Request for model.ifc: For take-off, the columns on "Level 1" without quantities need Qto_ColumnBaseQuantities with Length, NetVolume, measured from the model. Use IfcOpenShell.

First a look at what the model holds.

```python
import ifcopenshell
import ifcopenshell.util.element
import ifcopenshell.util.unit

model = ifcopenshell.open("model.ifc")
print(model.schema)
for unit_type in ("LENGTHUNIT", "AREAUNIT", "VOLUMEUNIT"):
    print(unit_type, ifcopenshell.util.unit.calculate_unit_scale(model, unit_type))
storey = next(s for s in model.by_type("IfcBuildingStorey") if s.Name == "Level 1")
columns = [e for e in ifcopenshell.util.element.get_decomposition(storey) if e.is_a("IfcColumn")]
for e in sorted(columns, key=lambda e: e.id()):
    print(e.id(), e.is_a(), e.Name, list(ifcopenshell.util.element.get_psets(e, qtos_only=True)), sep=" | ")
```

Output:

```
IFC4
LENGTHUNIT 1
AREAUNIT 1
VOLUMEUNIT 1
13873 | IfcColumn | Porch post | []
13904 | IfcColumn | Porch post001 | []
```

```python
import ifcopenshell
import ifcopenshell.api.pset
import ifcopenshell.geom
import ifcopenshell.util.element
import ifcopenshell.util.shape
import ifcopenshell.util.unit

model = ifcopenshell.open("model.ifc")
unit_scale = ifcopenshell.util.unit.calculate_unit_scale(model)
volume_scale = ifcopenshell.util.unit.calculate_unit_scale(model, "VOLUMEUNIT")
settings = ifcopenshell.geom.settings()

storey = next(s for s in model.by_type("IfcBuildingStorey") if s.Name == "Level 1")
columns = [e for e in ifcopenshell.util.element.get_decomposition(storey) if e.is_a("IfcColumn")]

for e in sorted(columns, key=lambda e: e.id()):
    if ifcopenshell.util.element.get_psets(e, qtos_only=True, should_inherit=False):
        continue
    # Geometry comes back in metres, in the element's own axes.
    shape = ifcopenshell.geom.create_shape(settings, e)
    values = {
        "Length": ifcopenshell.util.shape.get_z(shape.geometry) / unit_scale,
        "NetVolume": ifcopenshell.util.shape.get_volume(shape.geometry) / volume_scale,
    }
    qto = ifcopenshell.api.pset.add_qto(model, product=e, name="Qto_ColumnBaseQuantities")
    ifcopenshell.api.pset.edit_qto(model, qto=qto, properties=values)
    print(e.id(), {k: round(v, 3) for k, v in values.items()})

model.write("model_v2.ifc")
```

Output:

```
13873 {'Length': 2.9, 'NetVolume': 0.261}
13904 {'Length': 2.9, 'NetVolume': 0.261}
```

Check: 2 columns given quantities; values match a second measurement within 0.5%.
